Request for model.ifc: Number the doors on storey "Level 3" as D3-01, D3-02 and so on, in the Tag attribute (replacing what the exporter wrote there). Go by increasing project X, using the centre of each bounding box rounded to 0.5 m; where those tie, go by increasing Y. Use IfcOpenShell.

First a look at what the model holds.

```python
import ifcopenshell
import ifcopenshell.util.element
import ifcopenshell.util.placement

model = ifcopenshell.open("model.ifc")
print(model.schema)
storey = next(s for s in model.by_type("IfcBuildingStorey") if s.Name == "Level 3")
doors = [e for e in ifcopenshell.util.element.get_decomposition(storey) if e.is_a("IfcDoor")]
for e in sorted(doors, key=lambda e: e.id()):
    origin = ifcopenshell.util.placement.get_local_placement(e.ObjectPlacement)[:3, 3]
    print(e.id(), e.Tag, e.Name, origin.round(2) + 0.0, sep=" | ")
```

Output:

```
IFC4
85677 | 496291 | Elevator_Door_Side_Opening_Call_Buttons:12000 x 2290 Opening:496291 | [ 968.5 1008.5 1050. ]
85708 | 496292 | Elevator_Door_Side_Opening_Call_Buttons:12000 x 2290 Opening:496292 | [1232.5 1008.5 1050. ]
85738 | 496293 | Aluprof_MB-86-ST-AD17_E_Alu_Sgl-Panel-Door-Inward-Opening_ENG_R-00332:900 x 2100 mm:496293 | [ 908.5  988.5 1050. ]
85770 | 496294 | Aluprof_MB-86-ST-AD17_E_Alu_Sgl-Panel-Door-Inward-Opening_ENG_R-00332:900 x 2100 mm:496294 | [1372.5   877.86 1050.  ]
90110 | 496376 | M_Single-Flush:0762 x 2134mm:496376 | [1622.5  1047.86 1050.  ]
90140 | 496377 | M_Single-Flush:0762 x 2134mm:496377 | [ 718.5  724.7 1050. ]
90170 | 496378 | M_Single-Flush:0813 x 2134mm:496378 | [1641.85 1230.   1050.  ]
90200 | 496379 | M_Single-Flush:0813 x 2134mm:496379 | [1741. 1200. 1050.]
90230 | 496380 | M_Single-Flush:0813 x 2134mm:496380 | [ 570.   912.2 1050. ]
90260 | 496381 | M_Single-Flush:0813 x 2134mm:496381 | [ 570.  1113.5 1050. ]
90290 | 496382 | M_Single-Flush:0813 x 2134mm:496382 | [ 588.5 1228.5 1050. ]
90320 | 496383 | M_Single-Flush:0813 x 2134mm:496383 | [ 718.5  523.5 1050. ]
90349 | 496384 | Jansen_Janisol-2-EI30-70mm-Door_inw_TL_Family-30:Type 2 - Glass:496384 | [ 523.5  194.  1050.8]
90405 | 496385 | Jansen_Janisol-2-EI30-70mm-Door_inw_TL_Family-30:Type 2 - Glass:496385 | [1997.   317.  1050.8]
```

```python
import ifcopenshell
import ifcopenshell.geom
import ifcopenshell.util.element
import ifcopenshell.util.shape

model = ifcopenshell.open("model.ifc")
settings = ifcopenshell.geom.settings()
settings.set("use-world-coords", True)


def centre(element):
    shape = ifcopenshell.geom.create_shape(settings, element)
    return ifcopenshell.util.shape.get_bbox_centroid(shape.geometry)


storey = next(s for s in model.by_type("IfcBuildingStorey") if s.Name == "Level 3")
doors = [e for e in ifcopenshell.util.element.get_decomposition(storey) if e.is_a("IfcDoor")]

# Insertion points can sit at a corner or the storey origin, so sort by the geometry (in metres).
centres = {e: centre(e) for e in doors}
doors.sort(key=lambda e: (round(centres[e][0] / 0.5), centres[e][1]))

for i, e in enumerate(doors, start=1):
    number = f"D3-{i:02d}"
    e.Tag = number
    print(e.id(), number)

model.write("model_rev.ifc")
```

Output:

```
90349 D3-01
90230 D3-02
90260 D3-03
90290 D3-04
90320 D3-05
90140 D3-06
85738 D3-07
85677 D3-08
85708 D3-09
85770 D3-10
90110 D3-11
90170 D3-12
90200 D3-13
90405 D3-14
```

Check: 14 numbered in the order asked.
